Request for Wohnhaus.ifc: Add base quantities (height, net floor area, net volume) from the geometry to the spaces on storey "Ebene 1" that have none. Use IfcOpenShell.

First a look at what the model holds.

```python
import ifcopenshell
import ifcopenshell.util.element
import ifcopenshell.util.unit

model = ifcopenshell.open("Wohnhaus.ifc")
print(model.schema)
for unit_type in ("LENGTHUNIT", "AREAUNIT", "VOLUMEUNIT"):
    print(unit_type, ifcopenshell.util.unit.calculate_unit_scale(model, unit_type))
storey = next(s for s in model.by_type("IfcBuildingStorey") if s.Name == "Ebene 1")
spaces = [e for e in ifcopenshell.util.element.get_decomposition(storey) if e.is_a("IfcSpace")]
for e in sorted(spaces, key=lambda e: e.id()):
    print(e.id(), e.is_a(), e.Name, list(ifcopenshell.util.element.get_psets(e, qtos_only=True)), sep=" | ")
```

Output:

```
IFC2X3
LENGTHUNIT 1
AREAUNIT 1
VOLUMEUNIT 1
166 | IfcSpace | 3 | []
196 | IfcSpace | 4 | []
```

```python
import ifcopenshell
import ifcopenshell.api.pset
import ifcopenshell.geom
import ifcopenshell.util.element
import ifcopenshell.util.shape
import ifcopenshell.util.unit

model = ifcopenshell.open("Wohnhaus.ifc")
unit_scale = ifcopenshell.util.unit.calculate_unit_scale(model)
area_scale = ifcopenshell.util.unit.calculate_unit_scale(model, "AREAUNIT")
volume_scale = ifcopenshell.util.unit.calculate_unit_scale(model, "VOLUMEUNIT")
settings = ifcopenshell.geom.settings()

storey = next(s for s in model.by_type("IfcBuildingStorey") if s.Name == "Ebene 1")
spaces = [e for e in ifcopenshell.util.element.get_decomposition(storey) if e.is_a("IfcSpace")]

for e in sorted(spaces, key=lambda e: e.id()):
    if ifcopenshell.util.element.get_psets(e, qtos_only=True, should_inherit=False):
        continue
    # Geometry comes back in metres, in the element's own axes.
    shape = ifcopenshell.geom.create_shape(settings, e)
    values = {
        "Height": ifcopenshell.util.shape.get_z(shape.geometry) / unit_scale,
        "NetFloorArea": ifcopenshell.util.shape.get_footprint_area(shape.geometry) / area_scale,
        "NetVolume": ifcopenshell.util.shape.get_volume(shape.geometry) / volume_scale,
    }
    qto = ifcopenshell.api.pset.add_qto(model, product=e, name="BaseQuantities")
    ifcopenshell.api.pset.edit_qto(model, qto=qto, properties=values)
    print(e.id(), {k: round(v, 3) for k, v in values.items()})

model.write("Wohnhaus_updated.ifc")
```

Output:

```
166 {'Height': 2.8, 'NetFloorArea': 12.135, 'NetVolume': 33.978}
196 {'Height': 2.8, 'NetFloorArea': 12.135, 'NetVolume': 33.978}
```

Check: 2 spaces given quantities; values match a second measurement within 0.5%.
